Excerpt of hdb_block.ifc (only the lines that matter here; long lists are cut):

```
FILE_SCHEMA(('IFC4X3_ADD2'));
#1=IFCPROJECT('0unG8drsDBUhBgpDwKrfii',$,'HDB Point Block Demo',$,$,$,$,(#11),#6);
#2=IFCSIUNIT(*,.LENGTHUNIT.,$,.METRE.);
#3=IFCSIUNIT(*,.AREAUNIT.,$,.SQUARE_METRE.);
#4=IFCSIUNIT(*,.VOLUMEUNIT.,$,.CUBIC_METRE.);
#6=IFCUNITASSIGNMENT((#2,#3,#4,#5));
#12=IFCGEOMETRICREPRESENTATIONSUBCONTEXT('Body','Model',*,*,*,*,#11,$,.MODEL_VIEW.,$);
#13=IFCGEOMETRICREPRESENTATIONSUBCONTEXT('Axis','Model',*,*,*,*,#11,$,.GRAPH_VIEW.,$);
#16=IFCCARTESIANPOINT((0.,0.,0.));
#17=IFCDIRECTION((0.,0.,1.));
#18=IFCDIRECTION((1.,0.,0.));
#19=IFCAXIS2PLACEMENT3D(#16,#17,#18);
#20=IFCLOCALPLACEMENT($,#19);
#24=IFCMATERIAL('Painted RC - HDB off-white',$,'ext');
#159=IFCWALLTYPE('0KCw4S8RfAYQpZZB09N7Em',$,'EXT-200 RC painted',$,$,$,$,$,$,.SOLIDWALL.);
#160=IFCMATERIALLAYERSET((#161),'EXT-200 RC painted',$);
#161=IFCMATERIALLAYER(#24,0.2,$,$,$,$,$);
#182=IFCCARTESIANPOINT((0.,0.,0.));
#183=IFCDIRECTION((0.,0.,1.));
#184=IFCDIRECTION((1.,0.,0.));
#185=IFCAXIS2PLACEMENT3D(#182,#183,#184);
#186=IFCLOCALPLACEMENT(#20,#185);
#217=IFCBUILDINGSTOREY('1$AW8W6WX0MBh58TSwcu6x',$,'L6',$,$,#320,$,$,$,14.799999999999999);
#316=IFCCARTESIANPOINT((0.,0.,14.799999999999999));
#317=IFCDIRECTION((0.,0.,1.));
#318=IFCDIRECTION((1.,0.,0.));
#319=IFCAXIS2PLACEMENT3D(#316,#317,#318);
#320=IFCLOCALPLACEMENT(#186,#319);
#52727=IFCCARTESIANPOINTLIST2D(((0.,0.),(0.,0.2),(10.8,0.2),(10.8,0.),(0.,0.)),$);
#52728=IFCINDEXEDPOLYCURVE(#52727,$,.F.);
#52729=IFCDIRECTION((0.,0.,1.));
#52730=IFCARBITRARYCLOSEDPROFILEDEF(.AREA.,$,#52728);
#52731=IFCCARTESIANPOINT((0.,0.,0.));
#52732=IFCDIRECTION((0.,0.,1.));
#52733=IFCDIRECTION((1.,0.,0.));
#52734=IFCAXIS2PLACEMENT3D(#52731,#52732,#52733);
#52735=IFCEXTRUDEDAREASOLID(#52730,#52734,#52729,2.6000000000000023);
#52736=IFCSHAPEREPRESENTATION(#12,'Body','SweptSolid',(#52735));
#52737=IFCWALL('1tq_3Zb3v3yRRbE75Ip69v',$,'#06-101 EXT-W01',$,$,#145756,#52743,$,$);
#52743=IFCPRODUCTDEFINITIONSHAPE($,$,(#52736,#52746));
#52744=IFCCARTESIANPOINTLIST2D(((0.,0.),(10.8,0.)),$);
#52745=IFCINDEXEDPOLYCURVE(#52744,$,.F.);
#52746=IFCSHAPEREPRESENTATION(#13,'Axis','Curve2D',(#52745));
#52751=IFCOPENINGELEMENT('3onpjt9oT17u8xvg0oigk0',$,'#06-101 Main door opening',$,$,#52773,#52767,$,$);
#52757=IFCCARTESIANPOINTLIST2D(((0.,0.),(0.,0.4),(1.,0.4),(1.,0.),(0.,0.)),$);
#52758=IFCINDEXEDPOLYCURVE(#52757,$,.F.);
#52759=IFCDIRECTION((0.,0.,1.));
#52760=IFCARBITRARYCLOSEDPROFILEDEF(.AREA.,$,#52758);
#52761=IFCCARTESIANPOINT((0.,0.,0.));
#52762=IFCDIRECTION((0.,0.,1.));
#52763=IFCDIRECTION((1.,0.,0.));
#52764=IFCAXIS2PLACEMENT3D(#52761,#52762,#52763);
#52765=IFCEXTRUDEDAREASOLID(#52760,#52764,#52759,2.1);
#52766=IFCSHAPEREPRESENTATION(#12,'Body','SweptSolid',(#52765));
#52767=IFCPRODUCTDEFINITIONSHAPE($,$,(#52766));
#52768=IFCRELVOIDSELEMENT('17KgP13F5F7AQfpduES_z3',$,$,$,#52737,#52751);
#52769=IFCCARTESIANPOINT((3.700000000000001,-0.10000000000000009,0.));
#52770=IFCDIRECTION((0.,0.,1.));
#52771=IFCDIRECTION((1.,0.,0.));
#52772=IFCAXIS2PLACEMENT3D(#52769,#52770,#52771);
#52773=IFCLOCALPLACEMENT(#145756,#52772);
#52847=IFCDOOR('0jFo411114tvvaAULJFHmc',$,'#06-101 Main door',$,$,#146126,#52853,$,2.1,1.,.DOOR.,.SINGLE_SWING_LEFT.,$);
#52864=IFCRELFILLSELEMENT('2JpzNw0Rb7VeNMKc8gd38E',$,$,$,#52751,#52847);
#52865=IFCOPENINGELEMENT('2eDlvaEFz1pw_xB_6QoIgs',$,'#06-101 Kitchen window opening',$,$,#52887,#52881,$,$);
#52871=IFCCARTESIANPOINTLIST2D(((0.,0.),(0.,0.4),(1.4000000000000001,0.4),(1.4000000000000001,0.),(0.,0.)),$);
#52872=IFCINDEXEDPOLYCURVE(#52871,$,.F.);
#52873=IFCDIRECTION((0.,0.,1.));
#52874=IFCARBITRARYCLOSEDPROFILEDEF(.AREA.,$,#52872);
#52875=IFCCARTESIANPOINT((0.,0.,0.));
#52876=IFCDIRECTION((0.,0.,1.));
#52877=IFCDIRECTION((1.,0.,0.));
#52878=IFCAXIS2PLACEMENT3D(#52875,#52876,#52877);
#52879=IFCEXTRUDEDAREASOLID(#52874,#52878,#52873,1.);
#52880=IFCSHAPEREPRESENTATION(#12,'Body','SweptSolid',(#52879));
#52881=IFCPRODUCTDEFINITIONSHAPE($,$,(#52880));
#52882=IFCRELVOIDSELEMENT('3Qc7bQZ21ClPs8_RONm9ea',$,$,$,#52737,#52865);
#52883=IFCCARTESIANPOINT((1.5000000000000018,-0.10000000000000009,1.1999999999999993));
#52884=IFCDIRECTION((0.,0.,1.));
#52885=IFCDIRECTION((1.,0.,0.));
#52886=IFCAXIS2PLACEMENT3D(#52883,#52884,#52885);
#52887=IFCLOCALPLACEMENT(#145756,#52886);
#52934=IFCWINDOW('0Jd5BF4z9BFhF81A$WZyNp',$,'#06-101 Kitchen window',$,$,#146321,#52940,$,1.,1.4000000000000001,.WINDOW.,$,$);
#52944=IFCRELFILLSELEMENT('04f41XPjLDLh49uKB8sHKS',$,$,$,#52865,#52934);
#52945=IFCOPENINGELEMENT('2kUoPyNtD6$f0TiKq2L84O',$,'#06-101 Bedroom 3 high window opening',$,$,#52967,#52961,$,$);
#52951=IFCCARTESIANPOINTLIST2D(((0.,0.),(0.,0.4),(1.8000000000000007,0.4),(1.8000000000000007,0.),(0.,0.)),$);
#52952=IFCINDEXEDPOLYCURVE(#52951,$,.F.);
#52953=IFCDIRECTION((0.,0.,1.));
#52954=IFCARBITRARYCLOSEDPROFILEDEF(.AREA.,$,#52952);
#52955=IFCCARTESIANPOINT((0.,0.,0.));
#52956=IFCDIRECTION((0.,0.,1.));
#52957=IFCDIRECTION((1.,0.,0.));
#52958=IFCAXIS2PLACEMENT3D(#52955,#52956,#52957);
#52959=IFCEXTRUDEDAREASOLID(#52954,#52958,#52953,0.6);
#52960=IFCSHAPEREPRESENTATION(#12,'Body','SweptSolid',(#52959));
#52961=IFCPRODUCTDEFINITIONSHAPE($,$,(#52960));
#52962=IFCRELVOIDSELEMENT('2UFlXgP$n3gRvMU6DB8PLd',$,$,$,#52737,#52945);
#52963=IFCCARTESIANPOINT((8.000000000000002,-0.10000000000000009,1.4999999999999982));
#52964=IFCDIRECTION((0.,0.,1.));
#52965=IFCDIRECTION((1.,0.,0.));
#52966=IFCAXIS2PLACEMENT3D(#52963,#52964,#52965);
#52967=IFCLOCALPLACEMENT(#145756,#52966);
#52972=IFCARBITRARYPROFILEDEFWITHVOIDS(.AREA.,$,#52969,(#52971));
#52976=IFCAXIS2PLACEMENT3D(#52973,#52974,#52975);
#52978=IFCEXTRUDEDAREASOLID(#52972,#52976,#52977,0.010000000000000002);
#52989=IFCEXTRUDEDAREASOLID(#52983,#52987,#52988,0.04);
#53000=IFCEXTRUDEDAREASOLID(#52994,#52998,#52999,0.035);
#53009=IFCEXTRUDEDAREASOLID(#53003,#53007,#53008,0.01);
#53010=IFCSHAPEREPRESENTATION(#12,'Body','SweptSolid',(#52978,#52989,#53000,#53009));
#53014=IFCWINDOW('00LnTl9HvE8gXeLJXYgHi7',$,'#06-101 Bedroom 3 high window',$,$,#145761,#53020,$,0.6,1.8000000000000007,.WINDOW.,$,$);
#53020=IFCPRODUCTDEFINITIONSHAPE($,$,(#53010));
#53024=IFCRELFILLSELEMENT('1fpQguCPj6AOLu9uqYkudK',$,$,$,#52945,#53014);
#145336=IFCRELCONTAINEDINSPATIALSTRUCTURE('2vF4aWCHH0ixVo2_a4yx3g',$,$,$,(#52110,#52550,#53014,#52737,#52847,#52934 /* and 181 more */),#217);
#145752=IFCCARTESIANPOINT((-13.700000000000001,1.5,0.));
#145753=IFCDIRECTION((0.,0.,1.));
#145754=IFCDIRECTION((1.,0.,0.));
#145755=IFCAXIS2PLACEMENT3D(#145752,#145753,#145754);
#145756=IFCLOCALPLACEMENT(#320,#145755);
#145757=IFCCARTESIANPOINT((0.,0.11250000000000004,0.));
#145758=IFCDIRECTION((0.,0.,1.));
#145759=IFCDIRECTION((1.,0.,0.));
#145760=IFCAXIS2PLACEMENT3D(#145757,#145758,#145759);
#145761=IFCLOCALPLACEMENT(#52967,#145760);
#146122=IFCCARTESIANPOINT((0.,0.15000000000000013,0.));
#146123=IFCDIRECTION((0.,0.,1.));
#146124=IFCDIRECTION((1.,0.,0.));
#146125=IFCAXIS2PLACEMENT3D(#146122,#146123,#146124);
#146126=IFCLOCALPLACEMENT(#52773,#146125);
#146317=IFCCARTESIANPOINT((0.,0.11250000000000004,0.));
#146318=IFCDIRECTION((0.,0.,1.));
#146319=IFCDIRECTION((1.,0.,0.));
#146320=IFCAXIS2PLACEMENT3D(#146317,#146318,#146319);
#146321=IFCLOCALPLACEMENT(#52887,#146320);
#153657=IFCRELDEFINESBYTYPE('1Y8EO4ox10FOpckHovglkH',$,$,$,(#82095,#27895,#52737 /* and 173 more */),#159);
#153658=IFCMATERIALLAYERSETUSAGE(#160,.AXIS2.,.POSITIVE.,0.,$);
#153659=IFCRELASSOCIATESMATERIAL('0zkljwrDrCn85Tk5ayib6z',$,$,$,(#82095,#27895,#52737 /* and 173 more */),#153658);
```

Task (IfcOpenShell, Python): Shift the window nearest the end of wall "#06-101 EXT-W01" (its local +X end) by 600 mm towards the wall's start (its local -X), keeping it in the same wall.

```python
import ifcopenshell
import ifcopenshell.api.geometry
import ifcopenshell.util.placement

model = ifcopenshell.open("hdb_block.ifc")

window = model.by_guid("00LnTl9HvE8gXeLJXYgHi7")
opening = window.FillsVoids[0].RelatingOpeningElement
wall = opening.VoidsElements[0].RelatingBuildingElement

wall_matrix = ifcopenshell.util.placement.get_local_placement(wall.ObjectPlacement)
shift = wall_matrix[:3, 0] * -0.6
before = ifcopenshell.util.placement.get_local_placement(window.ObjectPlacement)[:3, 3].copy()

# The window is placed relative to its opening, so it follows when the opening moves.
matrix = ifcopenshell.util.placement.get_local_placement(opening.ObjectPlacement)
matrix[:3, 3] += shift
ifcopenshell.api.geometry.edit_object_placement(
    model, product=opening, matrix=matrix, is_si=False, should_transform_children=True
)

after = ifcopenshell.util.placement.get_local_placement(window.ObjectPlacement)[:3, 3]
print("window moved by", (after - before).round(3) + 0.0)

model.write("hdb_block_updated.ifc")
```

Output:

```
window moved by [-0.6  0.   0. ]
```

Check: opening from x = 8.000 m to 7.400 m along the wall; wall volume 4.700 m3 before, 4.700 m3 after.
